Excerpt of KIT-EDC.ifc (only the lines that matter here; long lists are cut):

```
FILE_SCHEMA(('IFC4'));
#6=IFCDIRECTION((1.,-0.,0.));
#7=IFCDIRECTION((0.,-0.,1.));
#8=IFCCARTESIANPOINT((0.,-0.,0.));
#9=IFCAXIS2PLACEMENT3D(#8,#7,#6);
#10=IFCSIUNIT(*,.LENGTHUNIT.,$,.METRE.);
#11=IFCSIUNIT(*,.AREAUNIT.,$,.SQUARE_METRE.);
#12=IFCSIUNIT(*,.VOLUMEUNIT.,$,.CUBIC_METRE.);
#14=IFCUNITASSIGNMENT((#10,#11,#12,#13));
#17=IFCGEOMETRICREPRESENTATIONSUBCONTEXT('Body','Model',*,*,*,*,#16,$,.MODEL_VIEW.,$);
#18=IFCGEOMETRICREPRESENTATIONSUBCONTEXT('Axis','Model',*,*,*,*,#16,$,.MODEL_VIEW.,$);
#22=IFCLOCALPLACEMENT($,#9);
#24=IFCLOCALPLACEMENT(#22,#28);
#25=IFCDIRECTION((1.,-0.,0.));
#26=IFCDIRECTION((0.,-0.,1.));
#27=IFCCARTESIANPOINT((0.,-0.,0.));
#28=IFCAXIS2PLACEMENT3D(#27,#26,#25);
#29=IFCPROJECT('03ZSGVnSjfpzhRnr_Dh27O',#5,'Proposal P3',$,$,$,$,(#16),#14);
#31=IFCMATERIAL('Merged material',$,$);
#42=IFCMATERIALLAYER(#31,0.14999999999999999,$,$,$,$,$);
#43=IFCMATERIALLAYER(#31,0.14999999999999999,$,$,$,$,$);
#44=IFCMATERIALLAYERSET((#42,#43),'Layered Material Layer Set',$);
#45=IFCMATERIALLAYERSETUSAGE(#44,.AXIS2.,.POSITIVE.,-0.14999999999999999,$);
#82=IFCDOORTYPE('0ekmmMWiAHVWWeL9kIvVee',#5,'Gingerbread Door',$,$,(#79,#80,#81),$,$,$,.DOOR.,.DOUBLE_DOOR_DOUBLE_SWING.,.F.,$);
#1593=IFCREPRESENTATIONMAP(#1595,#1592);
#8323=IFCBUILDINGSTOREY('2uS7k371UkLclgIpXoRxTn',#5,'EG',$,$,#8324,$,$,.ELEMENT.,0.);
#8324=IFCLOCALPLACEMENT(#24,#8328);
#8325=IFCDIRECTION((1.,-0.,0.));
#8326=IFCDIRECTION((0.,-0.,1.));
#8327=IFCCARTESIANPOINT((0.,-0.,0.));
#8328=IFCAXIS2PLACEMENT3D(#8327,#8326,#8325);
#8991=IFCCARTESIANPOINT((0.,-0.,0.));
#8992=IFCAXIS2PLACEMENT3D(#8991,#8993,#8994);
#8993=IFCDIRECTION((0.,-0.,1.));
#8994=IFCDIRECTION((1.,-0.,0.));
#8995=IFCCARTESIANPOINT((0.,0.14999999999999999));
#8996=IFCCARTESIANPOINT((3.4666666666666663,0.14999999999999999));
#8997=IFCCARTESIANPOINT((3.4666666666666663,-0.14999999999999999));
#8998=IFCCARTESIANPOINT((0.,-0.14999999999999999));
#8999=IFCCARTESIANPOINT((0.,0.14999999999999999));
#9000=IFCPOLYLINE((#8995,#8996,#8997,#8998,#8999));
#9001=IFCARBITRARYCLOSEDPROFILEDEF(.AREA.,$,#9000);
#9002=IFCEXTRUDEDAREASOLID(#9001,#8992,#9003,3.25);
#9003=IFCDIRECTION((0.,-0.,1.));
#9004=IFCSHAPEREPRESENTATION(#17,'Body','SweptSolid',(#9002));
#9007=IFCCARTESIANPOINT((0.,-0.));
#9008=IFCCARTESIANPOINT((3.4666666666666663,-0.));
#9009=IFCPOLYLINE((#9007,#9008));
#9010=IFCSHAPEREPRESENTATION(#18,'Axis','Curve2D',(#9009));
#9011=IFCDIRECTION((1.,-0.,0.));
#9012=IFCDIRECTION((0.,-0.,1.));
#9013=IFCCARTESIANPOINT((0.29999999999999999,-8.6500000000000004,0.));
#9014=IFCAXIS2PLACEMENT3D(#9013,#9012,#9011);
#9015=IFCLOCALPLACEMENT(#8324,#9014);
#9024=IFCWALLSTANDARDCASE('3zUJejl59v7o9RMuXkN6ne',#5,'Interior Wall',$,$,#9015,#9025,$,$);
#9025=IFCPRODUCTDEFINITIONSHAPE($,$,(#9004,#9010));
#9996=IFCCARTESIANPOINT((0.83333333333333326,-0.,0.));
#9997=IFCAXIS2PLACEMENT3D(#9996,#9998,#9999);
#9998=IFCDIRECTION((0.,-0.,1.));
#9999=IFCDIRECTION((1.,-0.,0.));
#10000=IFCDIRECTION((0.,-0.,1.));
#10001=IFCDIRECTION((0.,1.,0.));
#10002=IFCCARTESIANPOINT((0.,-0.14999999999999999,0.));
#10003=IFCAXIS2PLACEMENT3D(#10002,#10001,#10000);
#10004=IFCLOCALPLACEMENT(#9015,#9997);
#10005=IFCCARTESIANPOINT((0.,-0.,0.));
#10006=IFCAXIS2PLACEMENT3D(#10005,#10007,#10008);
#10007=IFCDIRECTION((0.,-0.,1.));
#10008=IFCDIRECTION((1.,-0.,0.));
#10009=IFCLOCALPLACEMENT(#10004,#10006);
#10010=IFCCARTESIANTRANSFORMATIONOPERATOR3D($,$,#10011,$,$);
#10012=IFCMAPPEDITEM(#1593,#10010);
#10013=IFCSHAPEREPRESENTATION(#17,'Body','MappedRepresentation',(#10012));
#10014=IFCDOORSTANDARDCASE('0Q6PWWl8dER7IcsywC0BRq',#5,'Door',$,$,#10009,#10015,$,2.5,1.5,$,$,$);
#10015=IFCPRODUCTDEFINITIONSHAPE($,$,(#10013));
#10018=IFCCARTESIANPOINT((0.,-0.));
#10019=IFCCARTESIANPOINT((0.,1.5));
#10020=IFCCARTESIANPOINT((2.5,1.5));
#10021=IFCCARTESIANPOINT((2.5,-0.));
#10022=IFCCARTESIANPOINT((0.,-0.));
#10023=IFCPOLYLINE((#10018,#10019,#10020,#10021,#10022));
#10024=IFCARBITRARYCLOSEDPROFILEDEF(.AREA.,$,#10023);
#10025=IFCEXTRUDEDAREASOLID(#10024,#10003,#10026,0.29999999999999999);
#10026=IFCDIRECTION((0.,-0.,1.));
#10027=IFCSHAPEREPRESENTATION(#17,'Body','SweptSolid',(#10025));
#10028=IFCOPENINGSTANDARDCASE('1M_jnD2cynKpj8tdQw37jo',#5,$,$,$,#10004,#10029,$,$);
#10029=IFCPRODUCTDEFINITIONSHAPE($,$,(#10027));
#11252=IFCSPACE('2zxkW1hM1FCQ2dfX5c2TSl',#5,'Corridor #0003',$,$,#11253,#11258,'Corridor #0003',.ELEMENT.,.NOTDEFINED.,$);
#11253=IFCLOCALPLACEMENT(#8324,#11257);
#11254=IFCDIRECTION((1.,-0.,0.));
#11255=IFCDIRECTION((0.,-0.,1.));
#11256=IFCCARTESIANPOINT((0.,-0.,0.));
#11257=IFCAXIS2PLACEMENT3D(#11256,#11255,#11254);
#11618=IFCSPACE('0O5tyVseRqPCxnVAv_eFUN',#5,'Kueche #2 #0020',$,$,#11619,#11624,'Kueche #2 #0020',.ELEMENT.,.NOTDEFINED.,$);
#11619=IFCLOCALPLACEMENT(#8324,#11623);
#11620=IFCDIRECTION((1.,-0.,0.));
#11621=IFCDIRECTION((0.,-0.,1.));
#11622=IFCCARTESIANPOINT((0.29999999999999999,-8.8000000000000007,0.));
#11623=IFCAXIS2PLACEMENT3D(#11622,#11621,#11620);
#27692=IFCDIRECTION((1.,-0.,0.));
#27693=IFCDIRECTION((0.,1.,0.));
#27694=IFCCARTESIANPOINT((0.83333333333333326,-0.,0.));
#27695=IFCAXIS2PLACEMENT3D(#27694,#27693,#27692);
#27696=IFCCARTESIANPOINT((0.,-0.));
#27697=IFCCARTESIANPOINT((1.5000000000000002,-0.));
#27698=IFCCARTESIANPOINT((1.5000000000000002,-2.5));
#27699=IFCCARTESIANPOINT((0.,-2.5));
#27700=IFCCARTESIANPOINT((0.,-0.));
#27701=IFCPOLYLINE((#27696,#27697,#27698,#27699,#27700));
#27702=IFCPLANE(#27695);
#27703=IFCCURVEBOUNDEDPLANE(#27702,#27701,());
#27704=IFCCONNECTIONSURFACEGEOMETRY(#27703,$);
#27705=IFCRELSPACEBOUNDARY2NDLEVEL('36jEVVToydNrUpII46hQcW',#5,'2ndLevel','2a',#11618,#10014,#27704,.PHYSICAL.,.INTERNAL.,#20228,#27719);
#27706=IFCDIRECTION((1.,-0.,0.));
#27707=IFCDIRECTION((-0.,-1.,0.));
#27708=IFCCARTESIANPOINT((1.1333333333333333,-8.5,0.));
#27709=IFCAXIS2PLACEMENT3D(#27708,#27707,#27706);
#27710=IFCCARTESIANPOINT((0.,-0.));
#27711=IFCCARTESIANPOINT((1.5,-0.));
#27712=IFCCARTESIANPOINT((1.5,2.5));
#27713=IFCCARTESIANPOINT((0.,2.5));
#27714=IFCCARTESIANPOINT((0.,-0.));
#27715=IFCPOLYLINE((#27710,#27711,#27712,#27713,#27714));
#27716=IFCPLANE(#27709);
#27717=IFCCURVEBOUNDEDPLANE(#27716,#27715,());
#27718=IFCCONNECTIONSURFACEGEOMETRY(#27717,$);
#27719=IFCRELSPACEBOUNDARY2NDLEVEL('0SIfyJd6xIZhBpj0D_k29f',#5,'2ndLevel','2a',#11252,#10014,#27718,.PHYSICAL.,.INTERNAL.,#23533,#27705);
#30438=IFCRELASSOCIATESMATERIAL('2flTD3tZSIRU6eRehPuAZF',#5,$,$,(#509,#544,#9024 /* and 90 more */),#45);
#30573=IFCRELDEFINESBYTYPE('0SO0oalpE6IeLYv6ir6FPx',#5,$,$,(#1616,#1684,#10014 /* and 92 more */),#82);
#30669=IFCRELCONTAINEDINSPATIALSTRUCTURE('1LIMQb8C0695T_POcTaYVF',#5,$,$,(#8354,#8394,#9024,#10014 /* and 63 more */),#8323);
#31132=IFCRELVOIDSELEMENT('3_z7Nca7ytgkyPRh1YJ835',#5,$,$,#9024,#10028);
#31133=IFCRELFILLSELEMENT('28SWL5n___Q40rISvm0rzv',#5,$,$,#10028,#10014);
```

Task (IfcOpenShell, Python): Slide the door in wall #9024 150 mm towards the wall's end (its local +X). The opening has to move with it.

```python
import numpy as np
import ifcopenshell
import ifcopenshell.api.geometry
import ifcopenshell.util.placement

model = ifcopenshell.open("KIT-EDC.ifc")

door = model.by_id(10014)
opening = door.FillsVoids[0].RelatingOpeningElement
wall = opening.VoidsElements[0].RelatingBuildingElement

wall_matrix = ifcopenshell.util.placement.get_local_placement(wall.ObjectPlacement)
shift = wall_matrix[:3, 0] * 0.15
before = ifcopenshell.util.placement.get_local_placement(door.ObjectPlacement)[:3, 3].copy()

# The door is placed relative to its opening, so it follows when the opening moves.
matrix = ifcopenshell.util.placement.get_local_placement(opening.ObjectPlacement)
matrix[:3, 3] += shift
ifcopenshell.api.geometry.edit_object_placement(
    model, product=opening, matrix=matrix, is_si=False, should_transform_children=True
)

# Space boundary surfaces are stored in each space's coordinates; move them too.
for rel in door.ProvidesBoundaries:
    if not rel.ConnectionGeometry:
        continue
    surface = rel.ConnectionGeometry.SurfaceOnRelatingElement.BasisSurface
    space_matrix = ifcopenshell.util.placement.get_local_placement(rel.RelatingSpace.ObjectPlacement)
    point = np.array(surface.Position.Location.Coordinates) + space_matrix[:3, :3].T @ shift
    surface.Position = model.createIfcAxis2Placement3D(
        model.createIfcCartesianPoint(point.tolist()), surface.Position.Axis, surface.Position.RefDirection
    )

after = ifcopenshell.util.placement.get_local_placement(door.ObjectPlacement)[:3, 3]
print("door moved by", (after - before).round(3) + 0.0)

model.write("KIT-EDC_v2.ifc")
```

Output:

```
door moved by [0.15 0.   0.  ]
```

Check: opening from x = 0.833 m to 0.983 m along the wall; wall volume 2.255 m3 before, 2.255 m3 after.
